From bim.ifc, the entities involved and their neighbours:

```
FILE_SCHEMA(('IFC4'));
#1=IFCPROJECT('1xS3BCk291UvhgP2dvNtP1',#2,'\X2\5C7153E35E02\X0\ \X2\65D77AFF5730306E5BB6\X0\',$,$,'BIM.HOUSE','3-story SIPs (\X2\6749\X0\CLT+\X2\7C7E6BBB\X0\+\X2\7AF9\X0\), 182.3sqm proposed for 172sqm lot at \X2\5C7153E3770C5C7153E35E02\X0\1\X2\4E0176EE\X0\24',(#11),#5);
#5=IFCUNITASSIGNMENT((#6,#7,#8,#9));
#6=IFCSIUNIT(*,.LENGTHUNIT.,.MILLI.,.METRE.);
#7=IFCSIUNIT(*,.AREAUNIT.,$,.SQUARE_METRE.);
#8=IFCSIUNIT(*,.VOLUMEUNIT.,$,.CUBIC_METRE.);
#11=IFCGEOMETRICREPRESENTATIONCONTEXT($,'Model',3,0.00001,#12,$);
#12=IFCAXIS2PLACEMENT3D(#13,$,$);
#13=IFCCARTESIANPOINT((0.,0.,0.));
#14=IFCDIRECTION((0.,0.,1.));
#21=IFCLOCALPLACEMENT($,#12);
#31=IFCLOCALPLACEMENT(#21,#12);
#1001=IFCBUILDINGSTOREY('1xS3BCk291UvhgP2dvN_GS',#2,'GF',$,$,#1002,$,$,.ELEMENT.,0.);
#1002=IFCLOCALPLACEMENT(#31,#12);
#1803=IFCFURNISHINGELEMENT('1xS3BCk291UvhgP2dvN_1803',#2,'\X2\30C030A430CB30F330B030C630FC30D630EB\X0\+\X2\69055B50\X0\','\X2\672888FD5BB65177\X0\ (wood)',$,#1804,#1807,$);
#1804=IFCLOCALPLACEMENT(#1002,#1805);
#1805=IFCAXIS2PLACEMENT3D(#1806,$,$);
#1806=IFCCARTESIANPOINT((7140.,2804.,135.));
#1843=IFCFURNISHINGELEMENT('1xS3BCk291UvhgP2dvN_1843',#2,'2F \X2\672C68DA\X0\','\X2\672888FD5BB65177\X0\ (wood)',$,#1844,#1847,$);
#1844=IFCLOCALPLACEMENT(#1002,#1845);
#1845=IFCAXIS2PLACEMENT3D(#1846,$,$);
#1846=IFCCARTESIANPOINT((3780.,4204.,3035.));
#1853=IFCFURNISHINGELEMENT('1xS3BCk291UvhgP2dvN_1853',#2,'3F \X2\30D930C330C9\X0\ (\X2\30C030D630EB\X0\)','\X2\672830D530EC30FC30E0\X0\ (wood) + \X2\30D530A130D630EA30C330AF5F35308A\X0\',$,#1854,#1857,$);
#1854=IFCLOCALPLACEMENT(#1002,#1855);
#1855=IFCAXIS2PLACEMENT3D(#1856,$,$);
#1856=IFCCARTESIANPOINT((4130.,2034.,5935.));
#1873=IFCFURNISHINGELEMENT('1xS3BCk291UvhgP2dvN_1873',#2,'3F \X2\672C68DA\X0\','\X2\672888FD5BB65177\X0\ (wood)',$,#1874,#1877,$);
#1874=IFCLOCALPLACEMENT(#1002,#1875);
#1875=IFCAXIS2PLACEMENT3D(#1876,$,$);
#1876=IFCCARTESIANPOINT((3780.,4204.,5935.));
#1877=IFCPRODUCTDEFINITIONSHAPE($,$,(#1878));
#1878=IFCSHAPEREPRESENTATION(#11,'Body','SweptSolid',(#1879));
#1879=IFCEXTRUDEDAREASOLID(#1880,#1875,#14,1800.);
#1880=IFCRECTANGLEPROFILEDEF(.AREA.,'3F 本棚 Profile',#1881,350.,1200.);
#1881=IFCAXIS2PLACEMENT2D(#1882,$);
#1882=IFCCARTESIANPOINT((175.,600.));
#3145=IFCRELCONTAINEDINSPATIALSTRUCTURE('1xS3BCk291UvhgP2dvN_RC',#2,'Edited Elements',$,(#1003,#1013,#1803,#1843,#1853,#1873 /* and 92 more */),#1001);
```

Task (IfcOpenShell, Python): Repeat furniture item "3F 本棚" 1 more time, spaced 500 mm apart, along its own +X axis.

```python
import ifcopenshell
import ifcopenshell.api.geometry
import ifcopenshell.api.root
import ifcopenshell.util.element
import ifcopenshell.util.placement
import ifcopenshell.util.unit

model = ifcopenshell.open("bim.ifc")
unit_scale = ifcopenshell.util.unit.calculate_unit_scale(model)


def reuse_history(source, copy):
    """copy_class also copies each property set's owner history, people and application; keep the originals."""
    for rel in copy.IsDefinedBy:
        if rel.is_a("IfcRelDefinesByProperties") and (history := rel.RelatingPropertyDefinition.OwnerHistory):
            rel.RelatingPropertyDefinition.OwnerHistory = source.OwnerHistory
            ifcopenshell.util.element.remove_deep2(model, history)


source = model.by_id(1873)
base = ifcopenshell.util.placement.get_local_placement(source.ObjectPlacement)
step = base[:3, 0] * 0.5 / unit_scale

for i in range(1, 2):
    copy = ifcopenshell.api.root.copy_class(model, product=source)
    copy.Representation = ifcopenshell.util.element.copy_deep(
        model, source.Representation, exclude=["IfcGeometricRepresentationContext", "IfcRepresentationMap"]
    )
    reuse_history(source, copy)
    matrix = base.copy()
    matrix[:3, 3] += i * step
    print("added at", matrix[:3, 3].round(3) + 0.0)
    ifcopenshell.api.geometry.edit_object_placement(model, product=copy, matrix=matrix, is_si=False)

model.write("bim-out.ifc")
```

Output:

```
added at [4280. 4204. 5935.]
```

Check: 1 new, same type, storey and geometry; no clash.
